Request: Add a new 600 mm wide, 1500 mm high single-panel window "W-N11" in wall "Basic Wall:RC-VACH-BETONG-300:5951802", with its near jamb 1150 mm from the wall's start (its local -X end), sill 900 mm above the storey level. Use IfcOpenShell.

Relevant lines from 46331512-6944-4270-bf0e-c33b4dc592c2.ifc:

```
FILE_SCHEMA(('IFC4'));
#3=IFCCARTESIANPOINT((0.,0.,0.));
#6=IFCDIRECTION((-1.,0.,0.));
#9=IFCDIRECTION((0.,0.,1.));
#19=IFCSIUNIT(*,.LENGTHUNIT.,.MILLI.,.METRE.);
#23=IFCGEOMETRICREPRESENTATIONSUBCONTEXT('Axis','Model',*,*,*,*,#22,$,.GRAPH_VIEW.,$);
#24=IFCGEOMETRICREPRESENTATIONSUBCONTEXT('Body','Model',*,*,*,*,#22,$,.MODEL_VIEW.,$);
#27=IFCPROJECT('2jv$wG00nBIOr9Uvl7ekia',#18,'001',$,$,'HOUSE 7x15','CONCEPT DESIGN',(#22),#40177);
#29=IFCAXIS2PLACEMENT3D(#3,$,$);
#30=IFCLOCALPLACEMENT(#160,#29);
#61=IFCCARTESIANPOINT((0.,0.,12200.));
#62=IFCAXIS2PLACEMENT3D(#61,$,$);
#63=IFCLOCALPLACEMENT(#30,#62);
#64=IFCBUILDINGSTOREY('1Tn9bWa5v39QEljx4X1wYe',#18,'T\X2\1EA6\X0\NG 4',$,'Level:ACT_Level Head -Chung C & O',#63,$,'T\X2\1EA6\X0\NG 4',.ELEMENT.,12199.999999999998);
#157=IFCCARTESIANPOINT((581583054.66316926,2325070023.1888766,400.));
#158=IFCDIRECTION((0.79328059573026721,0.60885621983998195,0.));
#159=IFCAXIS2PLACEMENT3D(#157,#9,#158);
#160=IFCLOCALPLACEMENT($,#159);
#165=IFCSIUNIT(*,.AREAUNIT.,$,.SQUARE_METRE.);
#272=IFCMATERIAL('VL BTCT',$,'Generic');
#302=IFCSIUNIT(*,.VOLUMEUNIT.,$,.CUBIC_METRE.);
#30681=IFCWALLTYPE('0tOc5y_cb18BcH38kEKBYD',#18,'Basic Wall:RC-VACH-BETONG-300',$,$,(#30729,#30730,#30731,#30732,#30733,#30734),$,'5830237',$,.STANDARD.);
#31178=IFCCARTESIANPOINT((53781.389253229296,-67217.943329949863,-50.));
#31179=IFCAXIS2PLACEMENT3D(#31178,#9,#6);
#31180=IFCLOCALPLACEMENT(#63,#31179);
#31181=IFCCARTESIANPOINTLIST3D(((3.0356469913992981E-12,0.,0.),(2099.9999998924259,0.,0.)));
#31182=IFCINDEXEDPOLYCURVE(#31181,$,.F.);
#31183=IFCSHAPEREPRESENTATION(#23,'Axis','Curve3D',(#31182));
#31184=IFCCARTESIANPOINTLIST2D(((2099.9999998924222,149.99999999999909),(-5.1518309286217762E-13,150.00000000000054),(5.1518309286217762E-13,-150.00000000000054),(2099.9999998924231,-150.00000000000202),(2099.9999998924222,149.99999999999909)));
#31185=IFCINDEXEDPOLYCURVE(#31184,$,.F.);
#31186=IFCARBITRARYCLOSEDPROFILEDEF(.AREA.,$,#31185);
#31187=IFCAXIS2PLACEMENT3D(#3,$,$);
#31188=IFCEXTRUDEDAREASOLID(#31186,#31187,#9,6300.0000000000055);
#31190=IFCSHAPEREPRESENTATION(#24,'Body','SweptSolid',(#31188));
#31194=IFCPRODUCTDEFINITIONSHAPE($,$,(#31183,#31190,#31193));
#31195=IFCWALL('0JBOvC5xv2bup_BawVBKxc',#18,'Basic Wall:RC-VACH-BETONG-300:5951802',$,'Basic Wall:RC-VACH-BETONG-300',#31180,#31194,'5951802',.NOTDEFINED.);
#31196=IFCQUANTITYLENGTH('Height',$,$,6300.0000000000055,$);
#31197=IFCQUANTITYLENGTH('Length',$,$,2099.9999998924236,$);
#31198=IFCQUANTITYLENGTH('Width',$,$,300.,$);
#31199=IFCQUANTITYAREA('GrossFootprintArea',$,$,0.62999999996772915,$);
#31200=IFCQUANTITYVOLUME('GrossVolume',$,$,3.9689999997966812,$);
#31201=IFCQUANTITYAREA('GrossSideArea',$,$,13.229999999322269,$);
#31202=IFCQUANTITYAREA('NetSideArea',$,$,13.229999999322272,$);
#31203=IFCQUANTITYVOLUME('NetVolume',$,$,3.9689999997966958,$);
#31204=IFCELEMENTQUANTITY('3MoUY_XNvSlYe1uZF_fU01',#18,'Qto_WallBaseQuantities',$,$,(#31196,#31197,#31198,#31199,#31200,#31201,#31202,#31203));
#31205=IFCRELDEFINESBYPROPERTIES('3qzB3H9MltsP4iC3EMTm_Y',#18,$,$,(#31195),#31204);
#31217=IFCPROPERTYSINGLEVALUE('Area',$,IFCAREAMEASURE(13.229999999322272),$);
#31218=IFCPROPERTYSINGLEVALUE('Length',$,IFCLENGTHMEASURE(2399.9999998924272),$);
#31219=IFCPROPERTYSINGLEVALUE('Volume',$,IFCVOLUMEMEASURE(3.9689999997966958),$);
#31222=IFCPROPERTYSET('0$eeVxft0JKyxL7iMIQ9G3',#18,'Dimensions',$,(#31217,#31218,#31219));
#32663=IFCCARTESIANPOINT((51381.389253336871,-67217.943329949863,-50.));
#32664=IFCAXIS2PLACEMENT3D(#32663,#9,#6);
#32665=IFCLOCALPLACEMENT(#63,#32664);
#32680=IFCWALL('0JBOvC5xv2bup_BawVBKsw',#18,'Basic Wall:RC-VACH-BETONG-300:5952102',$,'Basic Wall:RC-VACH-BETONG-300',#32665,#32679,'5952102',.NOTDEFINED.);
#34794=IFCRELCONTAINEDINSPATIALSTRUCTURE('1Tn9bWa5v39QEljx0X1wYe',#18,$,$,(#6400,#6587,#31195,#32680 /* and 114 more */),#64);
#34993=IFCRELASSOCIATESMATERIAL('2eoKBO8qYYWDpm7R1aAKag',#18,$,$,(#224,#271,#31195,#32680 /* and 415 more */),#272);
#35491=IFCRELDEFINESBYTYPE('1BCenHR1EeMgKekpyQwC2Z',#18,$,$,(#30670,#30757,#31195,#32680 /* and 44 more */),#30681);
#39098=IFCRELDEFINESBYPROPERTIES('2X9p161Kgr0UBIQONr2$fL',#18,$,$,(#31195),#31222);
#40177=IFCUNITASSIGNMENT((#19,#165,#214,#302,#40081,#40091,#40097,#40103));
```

```python
import numpy as np
import ifcopenshell
import ifcopenshell.api.feature
import ifcopenshell.api.geometry
import ifcopenshell.api.pset
import ifcopenshell.api.root
import ifcopenshell.api.spatial
import ifcopenshell.geom
import ifcopenshell.util.element
import ifcopenshell.util.placement
import ifcopenshell.util.representation
import ifcopenshell.util.shape
import ifcopenshell.util.unit

model = ifcopenshell.open("46331512-6944-4270-bf0e-c33b4dc592c2.ifc")
unit_scale = ifcopenshell.util.unit.calculate_unit_scale(model)
area_scale = ifcopenshell.util.unit.calculate_unit_scale(model, "AREAUNIT")
volume_scale = ifcopenshell.util.unit.calculate_unit_scale(model, "VOLUMEUNIT")
settings = ifcopenshell.geom.settings()


def volume(element):
    """Net volume in cubic metres, openings subtracted."""
    shape = ifcopenshell.geom.create_shape(settings, element)
    return ifcopenshell.util.shape.get_volume(shape.geometry)


wall = model.by_guid("0JBOvC5xv2bup_BawVBKxc")
storey = ifcopenshell.util.element.get_container(wall, ifc_class="IfcBuildingStorey")
context = ifcopenshell.util.representation.get_context(model, "Model", "Body", "MODEL_VIEW")
before = volume(wall)

width, height, from_end, sill = 0.6, 1.5, 1.15, 0.9  # metres

# The wall runs along its own X axis, and the end named is its -X end.
wall_shape = ifcopenshell.geom.create_shape(settings, wall)
x, y, z = ifcopenshell.util.shape.get_vertices(wall_shape.geometry).T
start = x.min() + from_end
face, thickness = float(y.min()), float(y.max() - y.min())
wall_matrix = ifcopenshell.util.placement.get_local_placement(wall.ObjectPlacement)
level = ifcopenshell.util.placement.get_local_placement(storey.ObjectPlacement)[2, 3]


def in_wall(x, y):
    """Placement at x, y metres in the wall's axes, at sill height."""
    matrix = wall_matrix.copy()
    matrix[:, 3] = wall_matrix @ np.array([x / unit_scale, y / unit_scale, 0.0, 1.0])
    matrix[2, 3] = level + sill / unit_scale
    return matrix


# Opening: a box that overshoots both wall faces by 50 mm.
opening = ifcopenshell.api.root.create_entity(model, ifc_class="IfcOpeningElement", predefined_type="OPENING")
box = ifcopenshell.api.geometry.add_wall_representation(
    model, context=context, length=width, height=height, thickness=thickness + 0.1
)
ifcopenshell.api.geometry.assign_representation(model, product=opening, representation=box)
ifcopenshell.api.geometry.edit_object_placement(model, product=opening, matrix=in_wall(start, face - 0.05), is_si=False)
ifcopenshell.api.feature.add_feature(model, feature=opening, element=wall)

window = ifcopenshell.api.root.create_entity(model, ifc_class="IfcWindow", name="W-N11", predefined_type="WINDOW")
window.OverallWidth, window.OverallHeight = width / unit_scale, height / unit_scale
window.PartitioningType = "SINGLE_PANEL"
body = ifcopenshell.api.geometry.add_window_representation(
    model,
    context=context,
    overall_width=window.OverallWidth,
    overall_height=window.OverallHeight,
    partition_type="SINGLE_PANEL",
)
ifcopenshell.api.geometry.assign_representation(model, product=window, representation=body)
ifcopenshell.api.spatial.assign_container(model, products=[window], relating_structure=storey)
ifcopenshell.api.feature.add_filling(model, opening=opening, element=window)

# Centre the window in the wall's thickness.
ifcopenshell.api.geometry.edit_object_placement(model, product=window, matrix=in_wall(start, face), is_si=False)
window_shape = ifcopenshell.geom.create_shape(settings, window)
depth = ifcopenshell.util.shape.get_vertices(window_shape.geometry)[:, 1]
offset = face + thickness / 2 - (depth.min() + depth.max()) / 2
ifcopenshell.api.geometry.edit_object_placement(model, product=window, matrix=in_wall(start, offset), is_si=False)

after = volume(wall)

# Update the wall's stored quantities.
qto = model.by_id(ifcopenshell.util.element.get_pset(wall, "Qto_WallBaseQuantities", should_inherit=False)["id"])
ifcopenshell.api.pset.edit_qto(model, qto=qto, properties={
    "NetSideArea": after / thickness / area_scale,
    "NetVolume": after / volume_scale,
})
pset = model.by_id(ifcopenshell.util.element.get_pset(wall, "Dimensions", should_inherit=False)["id"])
ifcopenshell.api.pset.edit_pset(model, pset=pset, properties={
    "Area": model.create_entity("IfcAreaMeasure", after / thickness / area_scale),
    "Volume": model.create_entity("IfcVolumeMeasure", after / volume_scale),
})

print(f"wall volume {before:.3f} -> {after:.3f} m3")

model.write("46331512-6944-4270-bf0e-c33b4dc592c2_rev.ifc")
```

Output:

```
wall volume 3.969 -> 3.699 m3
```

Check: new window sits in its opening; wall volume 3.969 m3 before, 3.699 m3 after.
